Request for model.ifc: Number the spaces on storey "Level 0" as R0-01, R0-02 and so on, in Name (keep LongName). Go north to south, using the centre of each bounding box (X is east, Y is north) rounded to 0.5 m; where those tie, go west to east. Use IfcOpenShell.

First a look at what the model holds.

```python
import ifcopenshell
import ifcopenshell.util.element
import ifcopenshell.util.placement

model = ifcopenshell.open("model.ifc")
print(model.schema)
storey = next(s for s in model.by_type("IfcBuildingStorey") if s.Name == "Level 0")
spaces = [e for e in ifcopenshell.util.element.get_decomposition(storey) if e.is_a("IfcSpace")]
for e in sorted(spaces, key=lambda e: e.id()):
    origin = ifcopenshell.util.placement.get_local_placement(e.ObjectPlacement)[:3, 3]
    print(e.id(), e.Name, e.LongName, origin.round(2) + 0.0, sep=" | ")
```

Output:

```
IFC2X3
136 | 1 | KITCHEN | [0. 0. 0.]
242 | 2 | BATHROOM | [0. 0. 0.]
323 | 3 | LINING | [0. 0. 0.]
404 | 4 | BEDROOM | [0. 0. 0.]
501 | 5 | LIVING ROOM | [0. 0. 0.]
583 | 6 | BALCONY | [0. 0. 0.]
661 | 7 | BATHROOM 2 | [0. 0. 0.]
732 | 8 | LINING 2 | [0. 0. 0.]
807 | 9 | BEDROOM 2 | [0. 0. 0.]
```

```python
import ifcopenshell
import ifcopenshell.geom
import ifcopenshell.util.element
import ifcopenshell.util.shape

model = ifcopenshell.open("model.ifc")
settings = ifcopenshell.geom.settings()
settings.set("use-world-coords", True)


def centre(element):
    shape = ifcopenshell.geom.create_shape(settings, element)
    return ifcopenshell.util.shape.get_bbox_centroid(shape.geometry)


storey = next(s for s in model.by_type("IfcBuildingStorey") if s.Name == "Level 0")
spaces = [e for e in ifcopenshell.util.element.get_decomposition(storey) if e.is_a("IfcSpace")]

# Insertion points can sit at a corner or the storey origin, so sort by the geometry (in metres).
centres = {e: centre(e) for e in spaces}
spaces.sort(key=lambda e: (-round(centres[e][1] / 0.5), centres[e][0]))

for i, e in enumerate(spaces, start=1):
    number = f"R0-{i:02d}"
    e.Name = number
    print(e.id(), number)

model.write("model_v2.ifc")
```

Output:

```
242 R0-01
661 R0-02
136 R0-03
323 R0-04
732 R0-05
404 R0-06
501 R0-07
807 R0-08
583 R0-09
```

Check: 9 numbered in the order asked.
